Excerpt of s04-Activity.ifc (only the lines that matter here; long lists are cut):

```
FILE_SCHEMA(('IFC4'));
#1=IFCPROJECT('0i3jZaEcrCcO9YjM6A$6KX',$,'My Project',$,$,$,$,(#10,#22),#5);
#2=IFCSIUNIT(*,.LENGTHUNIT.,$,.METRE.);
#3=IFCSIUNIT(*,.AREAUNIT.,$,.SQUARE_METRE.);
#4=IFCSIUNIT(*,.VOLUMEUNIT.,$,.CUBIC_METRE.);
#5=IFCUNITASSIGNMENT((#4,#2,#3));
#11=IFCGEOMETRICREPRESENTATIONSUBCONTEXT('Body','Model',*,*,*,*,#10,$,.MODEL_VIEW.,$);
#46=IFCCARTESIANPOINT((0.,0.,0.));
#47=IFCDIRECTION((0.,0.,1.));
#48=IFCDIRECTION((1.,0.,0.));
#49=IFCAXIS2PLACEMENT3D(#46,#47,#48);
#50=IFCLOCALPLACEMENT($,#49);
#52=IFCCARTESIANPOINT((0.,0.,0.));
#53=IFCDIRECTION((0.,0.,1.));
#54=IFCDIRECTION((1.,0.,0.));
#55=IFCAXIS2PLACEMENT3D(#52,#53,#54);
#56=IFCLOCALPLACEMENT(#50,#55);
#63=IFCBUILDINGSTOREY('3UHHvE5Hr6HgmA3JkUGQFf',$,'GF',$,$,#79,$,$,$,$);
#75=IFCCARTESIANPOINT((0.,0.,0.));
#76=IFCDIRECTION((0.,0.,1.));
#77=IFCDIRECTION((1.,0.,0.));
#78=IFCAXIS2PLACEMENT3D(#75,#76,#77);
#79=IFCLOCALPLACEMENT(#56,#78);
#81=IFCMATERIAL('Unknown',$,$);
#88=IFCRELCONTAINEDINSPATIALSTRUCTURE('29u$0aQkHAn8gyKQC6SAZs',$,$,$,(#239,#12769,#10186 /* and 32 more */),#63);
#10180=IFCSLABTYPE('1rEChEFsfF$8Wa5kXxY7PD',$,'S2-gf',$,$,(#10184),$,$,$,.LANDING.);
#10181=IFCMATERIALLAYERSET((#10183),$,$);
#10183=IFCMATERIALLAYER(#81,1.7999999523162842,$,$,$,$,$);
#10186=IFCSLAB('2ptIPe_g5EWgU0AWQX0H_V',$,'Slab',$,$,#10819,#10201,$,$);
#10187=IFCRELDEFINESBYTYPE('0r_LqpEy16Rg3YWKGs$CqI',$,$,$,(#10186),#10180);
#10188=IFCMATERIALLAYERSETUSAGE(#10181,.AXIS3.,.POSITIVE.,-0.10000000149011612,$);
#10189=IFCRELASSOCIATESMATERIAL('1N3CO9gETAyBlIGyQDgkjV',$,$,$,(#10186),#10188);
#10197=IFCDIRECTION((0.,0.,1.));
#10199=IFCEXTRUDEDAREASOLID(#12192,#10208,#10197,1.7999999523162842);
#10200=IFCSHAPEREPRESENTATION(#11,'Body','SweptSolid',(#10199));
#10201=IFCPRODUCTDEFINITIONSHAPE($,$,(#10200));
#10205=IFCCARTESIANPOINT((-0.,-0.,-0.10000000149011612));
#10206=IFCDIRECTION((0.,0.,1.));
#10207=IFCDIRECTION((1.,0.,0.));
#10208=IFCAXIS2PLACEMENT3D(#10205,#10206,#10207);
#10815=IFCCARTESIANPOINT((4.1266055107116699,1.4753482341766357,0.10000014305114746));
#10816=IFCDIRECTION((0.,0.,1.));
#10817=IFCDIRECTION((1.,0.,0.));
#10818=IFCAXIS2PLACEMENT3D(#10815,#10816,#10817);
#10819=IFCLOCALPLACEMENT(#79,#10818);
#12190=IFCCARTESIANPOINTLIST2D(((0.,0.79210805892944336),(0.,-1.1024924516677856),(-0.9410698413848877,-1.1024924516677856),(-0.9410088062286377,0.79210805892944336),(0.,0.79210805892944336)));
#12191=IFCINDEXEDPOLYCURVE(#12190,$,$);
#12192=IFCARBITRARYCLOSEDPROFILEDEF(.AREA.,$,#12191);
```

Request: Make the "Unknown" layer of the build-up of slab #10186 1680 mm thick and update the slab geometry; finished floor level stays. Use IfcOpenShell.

```python
import ifcopenshell
import ifcopenshell.util.element
import ifcopenshell.util.representation
import ifcopenshell.util.unit

model = ifcopenshell.open("s04-Activity.ifc")
unit_scale = ifcopenshell.util.unit.calculate_unit_scale(model)

layer_set = model.by_id(10181)
layer = next(l for l in layer_set.MaterialLayers if l.Material and l.Material.Name == "Unknown")
change = 1.68 / unit_scale - layer.LayerThickness
layer.LayerThickness += change

# Geometry does not follow the layer set by itself.
slabs = [e for e in ifcopenshell.util.element.get_elements_by_material(model, layer_set) if e.is_a("IfcSlab")]
for slab in sorted(slabs, key=lambda e: e.id()):
    body = ifcopenshell.util.representation.get_representation(slab, "Model", "Body")
    solid = body.Items[0]
    old_depth = solid.Depth
    solid.Depth += change
    # Extruded upwards: lower the start of the extrusion so the top stays.
    x, y, z = solid.Position.Location.Coordinates
    solid.Position.Location = model.createIfcCartesianPoint((x, y, z - change))
    print(slab.id(), f"{old_depth:g} -> {solid.Depth:g}")

# The layers are counted up from the underside, which has moved.
for usage in {ifcopenshell.util.element.get_material(slab) for slab in slabs}:
    usage.OffsetFromReferenceLine -= change

model.write("s04-Activity_rev.ifc")
```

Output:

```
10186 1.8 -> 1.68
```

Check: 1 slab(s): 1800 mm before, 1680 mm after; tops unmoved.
